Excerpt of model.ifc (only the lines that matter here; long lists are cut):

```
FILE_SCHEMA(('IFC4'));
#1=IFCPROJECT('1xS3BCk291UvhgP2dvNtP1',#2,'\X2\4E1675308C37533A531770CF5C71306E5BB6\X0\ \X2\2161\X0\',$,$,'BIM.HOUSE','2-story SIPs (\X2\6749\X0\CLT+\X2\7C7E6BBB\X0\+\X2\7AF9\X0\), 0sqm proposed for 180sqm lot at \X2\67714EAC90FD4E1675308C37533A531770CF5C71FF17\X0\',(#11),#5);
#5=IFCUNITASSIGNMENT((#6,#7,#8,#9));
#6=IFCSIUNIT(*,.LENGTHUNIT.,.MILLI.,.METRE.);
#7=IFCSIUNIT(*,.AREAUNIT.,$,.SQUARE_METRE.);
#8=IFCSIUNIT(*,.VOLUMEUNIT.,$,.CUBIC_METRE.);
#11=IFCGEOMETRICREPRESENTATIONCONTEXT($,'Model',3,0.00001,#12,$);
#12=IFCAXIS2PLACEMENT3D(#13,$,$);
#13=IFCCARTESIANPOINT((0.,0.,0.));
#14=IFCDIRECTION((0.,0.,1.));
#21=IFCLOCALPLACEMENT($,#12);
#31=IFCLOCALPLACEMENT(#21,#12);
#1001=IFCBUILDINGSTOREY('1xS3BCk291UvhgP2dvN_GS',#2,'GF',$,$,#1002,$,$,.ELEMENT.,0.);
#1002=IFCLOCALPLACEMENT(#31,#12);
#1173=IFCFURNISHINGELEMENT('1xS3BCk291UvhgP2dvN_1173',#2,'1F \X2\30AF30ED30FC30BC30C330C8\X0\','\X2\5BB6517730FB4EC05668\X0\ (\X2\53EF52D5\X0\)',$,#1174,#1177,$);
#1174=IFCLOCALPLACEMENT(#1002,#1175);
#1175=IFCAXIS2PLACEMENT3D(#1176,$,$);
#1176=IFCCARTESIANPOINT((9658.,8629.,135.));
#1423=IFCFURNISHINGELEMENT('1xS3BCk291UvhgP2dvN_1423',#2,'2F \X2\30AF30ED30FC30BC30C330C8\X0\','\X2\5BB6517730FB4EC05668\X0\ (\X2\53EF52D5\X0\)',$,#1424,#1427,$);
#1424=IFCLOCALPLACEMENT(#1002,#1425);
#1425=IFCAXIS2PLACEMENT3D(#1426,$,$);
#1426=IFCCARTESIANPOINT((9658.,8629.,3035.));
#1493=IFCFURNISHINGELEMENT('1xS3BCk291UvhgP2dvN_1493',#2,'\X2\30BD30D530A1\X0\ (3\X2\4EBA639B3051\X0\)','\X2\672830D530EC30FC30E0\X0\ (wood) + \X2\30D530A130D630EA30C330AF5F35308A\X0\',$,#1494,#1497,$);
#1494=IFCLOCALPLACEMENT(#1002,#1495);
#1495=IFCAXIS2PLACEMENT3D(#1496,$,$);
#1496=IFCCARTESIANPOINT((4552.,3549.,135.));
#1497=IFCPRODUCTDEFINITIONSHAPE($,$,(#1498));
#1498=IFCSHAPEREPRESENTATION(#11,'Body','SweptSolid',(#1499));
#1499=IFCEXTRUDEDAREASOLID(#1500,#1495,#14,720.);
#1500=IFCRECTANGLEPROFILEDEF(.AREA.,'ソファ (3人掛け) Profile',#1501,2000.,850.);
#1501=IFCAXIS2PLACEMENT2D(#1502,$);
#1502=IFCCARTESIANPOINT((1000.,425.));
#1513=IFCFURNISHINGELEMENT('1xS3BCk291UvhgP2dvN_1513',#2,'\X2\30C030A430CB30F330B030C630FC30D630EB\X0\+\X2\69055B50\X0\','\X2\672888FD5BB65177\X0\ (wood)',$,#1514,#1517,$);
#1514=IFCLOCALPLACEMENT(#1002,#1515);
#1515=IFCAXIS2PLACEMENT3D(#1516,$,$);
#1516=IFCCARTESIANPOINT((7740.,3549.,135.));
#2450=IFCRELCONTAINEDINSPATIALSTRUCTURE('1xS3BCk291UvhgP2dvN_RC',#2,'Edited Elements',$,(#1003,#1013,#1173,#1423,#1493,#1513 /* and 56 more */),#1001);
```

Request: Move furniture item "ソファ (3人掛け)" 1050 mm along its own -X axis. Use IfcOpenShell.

```python
import ifcopenshell
import ifcopenshell.api.geometry
import ifcopenshell.util.placement
import ifcopenshell.util.unit

model = ifcopenshell.open("model.ifc")
unit_scale = ifcopenshell.util.unit.calculate_unit_scale(model)

item = model.by_id(1493)
matrix = ifcopenshell.util.placement.get_local_placement(item.ObjectPlacement)
matrix[:3, 3] -= matrix[:3, 0] * 1.05 / unit_scale
ifcopenshell.api.geometry.edit_object_placement(model, product=item, matrix=matrix, is_si=False)

print(ifcopenshell.util.placement.get_local_placement(item.ObjectPlacement).round(3) + 0.0)

model.write("model_edited.ifc")
```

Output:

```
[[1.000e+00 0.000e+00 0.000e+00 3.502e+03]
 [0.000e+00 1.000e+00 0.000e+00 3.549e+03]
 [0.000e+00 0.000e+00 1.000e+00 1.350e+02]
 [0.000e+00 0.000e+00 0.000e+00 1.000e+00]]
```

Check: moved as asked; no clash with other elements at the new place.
